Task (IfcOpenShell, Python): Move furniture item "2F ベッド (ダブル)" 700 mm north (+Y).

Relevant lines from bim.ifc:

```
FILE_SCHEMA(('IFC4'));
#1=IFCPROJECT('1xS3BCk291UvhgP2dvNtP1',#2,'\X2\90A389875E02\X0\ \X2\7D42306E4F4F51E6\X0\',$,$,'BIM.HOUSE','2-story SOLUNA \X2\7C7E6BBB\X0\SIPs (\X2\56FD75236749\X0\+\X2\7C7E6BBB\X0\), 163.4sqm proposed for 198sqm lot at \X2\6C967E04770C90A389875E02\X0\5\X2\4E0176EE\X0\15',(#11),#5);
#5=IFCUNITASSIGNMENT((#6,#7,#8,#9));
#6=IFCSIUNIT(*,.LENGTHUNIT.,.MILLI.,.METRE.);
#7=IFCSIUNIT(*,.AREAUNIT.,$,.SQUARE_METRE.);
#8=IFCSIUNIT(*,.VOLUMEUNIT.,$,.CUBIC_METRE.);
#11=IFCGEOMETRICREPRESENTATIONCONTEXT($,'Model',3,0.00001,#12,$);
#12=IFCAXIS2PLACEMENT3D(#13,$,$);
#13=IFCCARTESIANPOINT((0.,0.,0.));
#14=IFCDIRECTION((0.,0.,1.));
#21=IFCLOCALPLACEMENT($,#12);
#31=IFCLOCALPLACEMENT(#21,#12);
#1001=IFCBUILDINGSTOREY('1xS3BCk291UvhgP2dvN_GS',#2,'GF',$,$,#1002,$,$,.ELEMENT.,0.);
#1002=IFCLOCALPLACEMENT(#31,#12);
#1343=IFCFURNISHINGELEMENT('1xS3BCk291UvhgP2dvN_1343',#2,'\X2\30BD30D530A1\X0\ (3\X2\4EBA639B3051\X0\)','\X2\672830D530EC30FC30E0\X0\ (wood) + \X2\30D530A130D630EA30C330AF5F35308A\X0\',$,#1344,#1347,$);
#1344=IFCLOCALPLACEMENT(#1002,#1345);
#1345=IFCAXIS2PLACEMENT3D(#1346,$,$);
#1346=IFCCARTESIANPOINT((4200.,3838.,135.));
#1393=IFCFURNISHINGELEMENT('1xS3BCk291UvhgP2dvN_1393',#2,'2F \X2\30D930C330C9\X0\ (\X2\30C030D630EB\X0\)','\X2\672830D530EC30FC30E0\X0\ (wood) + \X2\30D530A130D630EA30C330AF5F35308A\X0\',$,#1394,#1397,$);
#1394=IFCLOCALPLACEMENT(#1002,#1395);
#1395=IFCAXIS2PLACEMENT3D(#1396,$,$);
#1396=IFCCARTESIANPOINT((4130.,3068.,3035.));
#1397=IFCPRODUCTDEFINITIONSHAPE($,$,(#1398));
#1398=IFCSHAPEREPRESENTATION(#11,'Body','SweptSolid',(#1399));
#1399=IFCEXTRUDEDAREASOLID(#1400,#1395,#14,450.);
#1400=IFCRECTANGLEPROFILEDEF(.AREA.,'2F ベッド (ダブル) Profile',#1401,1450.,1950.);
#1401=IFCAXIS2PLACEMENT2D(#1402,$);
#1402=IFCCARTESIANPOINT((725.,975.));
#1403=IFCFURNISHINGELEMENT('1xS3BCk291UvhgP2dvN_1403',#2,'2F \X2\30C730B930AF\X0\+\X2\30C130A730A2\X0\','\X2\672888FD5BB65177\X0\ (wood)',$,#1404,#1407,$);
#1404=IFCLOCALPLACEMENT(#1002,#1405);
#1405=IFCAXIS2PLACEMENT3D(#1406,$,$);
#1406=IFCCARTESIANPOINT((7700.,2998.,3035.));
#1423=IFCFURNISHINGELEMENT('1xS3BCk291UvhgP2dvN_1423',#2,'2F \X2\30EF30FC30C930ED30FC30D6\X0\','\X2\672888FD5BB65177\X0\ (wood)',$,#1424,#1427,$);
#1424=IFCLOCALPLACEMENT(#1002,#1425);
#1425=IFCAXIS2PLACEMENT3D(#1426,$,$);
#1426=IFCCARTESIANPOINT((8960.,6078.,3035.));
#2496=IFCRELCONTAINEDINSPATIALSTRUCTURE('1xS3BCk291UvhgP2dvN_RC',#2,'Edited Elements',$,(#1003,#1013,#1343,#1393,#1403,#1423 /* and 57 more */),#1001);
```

```python
import ifcopenshell
import ifcopenshell.api.geometry
import ifcopenshell.util.placement
import ifcopenshell.util.unit

model = ifcopenshell.open("bim.ifc")
unit_scale = ifcopenshell.util.unit.calculate_unit_scale(model)

item = model.by_guid("1xS3BCk291UvhgP2dvN_1393")
matrix = ifcopenshell.util.placement.get_local_placement(item.ObjectPlacement)
matrix[1, 3] += 0.7 / unit_scale
ifcopenshell.api.geometry.edit_object_placement(model, product=item, matrix=matrix, is_si=False)

print(ifcopenshell.util.placement.get_local_placement(item.ObjectPlacement).round(3) + 0.0)

model.write("bim-out.ifc")
```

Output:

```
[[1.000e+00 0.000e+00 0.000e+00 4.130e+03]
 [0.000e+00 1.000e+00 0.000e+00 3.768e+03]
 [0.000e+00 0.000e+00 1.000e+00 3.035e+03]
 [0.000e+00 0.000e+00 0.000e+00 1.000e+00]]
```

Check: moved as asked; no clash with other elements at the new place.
